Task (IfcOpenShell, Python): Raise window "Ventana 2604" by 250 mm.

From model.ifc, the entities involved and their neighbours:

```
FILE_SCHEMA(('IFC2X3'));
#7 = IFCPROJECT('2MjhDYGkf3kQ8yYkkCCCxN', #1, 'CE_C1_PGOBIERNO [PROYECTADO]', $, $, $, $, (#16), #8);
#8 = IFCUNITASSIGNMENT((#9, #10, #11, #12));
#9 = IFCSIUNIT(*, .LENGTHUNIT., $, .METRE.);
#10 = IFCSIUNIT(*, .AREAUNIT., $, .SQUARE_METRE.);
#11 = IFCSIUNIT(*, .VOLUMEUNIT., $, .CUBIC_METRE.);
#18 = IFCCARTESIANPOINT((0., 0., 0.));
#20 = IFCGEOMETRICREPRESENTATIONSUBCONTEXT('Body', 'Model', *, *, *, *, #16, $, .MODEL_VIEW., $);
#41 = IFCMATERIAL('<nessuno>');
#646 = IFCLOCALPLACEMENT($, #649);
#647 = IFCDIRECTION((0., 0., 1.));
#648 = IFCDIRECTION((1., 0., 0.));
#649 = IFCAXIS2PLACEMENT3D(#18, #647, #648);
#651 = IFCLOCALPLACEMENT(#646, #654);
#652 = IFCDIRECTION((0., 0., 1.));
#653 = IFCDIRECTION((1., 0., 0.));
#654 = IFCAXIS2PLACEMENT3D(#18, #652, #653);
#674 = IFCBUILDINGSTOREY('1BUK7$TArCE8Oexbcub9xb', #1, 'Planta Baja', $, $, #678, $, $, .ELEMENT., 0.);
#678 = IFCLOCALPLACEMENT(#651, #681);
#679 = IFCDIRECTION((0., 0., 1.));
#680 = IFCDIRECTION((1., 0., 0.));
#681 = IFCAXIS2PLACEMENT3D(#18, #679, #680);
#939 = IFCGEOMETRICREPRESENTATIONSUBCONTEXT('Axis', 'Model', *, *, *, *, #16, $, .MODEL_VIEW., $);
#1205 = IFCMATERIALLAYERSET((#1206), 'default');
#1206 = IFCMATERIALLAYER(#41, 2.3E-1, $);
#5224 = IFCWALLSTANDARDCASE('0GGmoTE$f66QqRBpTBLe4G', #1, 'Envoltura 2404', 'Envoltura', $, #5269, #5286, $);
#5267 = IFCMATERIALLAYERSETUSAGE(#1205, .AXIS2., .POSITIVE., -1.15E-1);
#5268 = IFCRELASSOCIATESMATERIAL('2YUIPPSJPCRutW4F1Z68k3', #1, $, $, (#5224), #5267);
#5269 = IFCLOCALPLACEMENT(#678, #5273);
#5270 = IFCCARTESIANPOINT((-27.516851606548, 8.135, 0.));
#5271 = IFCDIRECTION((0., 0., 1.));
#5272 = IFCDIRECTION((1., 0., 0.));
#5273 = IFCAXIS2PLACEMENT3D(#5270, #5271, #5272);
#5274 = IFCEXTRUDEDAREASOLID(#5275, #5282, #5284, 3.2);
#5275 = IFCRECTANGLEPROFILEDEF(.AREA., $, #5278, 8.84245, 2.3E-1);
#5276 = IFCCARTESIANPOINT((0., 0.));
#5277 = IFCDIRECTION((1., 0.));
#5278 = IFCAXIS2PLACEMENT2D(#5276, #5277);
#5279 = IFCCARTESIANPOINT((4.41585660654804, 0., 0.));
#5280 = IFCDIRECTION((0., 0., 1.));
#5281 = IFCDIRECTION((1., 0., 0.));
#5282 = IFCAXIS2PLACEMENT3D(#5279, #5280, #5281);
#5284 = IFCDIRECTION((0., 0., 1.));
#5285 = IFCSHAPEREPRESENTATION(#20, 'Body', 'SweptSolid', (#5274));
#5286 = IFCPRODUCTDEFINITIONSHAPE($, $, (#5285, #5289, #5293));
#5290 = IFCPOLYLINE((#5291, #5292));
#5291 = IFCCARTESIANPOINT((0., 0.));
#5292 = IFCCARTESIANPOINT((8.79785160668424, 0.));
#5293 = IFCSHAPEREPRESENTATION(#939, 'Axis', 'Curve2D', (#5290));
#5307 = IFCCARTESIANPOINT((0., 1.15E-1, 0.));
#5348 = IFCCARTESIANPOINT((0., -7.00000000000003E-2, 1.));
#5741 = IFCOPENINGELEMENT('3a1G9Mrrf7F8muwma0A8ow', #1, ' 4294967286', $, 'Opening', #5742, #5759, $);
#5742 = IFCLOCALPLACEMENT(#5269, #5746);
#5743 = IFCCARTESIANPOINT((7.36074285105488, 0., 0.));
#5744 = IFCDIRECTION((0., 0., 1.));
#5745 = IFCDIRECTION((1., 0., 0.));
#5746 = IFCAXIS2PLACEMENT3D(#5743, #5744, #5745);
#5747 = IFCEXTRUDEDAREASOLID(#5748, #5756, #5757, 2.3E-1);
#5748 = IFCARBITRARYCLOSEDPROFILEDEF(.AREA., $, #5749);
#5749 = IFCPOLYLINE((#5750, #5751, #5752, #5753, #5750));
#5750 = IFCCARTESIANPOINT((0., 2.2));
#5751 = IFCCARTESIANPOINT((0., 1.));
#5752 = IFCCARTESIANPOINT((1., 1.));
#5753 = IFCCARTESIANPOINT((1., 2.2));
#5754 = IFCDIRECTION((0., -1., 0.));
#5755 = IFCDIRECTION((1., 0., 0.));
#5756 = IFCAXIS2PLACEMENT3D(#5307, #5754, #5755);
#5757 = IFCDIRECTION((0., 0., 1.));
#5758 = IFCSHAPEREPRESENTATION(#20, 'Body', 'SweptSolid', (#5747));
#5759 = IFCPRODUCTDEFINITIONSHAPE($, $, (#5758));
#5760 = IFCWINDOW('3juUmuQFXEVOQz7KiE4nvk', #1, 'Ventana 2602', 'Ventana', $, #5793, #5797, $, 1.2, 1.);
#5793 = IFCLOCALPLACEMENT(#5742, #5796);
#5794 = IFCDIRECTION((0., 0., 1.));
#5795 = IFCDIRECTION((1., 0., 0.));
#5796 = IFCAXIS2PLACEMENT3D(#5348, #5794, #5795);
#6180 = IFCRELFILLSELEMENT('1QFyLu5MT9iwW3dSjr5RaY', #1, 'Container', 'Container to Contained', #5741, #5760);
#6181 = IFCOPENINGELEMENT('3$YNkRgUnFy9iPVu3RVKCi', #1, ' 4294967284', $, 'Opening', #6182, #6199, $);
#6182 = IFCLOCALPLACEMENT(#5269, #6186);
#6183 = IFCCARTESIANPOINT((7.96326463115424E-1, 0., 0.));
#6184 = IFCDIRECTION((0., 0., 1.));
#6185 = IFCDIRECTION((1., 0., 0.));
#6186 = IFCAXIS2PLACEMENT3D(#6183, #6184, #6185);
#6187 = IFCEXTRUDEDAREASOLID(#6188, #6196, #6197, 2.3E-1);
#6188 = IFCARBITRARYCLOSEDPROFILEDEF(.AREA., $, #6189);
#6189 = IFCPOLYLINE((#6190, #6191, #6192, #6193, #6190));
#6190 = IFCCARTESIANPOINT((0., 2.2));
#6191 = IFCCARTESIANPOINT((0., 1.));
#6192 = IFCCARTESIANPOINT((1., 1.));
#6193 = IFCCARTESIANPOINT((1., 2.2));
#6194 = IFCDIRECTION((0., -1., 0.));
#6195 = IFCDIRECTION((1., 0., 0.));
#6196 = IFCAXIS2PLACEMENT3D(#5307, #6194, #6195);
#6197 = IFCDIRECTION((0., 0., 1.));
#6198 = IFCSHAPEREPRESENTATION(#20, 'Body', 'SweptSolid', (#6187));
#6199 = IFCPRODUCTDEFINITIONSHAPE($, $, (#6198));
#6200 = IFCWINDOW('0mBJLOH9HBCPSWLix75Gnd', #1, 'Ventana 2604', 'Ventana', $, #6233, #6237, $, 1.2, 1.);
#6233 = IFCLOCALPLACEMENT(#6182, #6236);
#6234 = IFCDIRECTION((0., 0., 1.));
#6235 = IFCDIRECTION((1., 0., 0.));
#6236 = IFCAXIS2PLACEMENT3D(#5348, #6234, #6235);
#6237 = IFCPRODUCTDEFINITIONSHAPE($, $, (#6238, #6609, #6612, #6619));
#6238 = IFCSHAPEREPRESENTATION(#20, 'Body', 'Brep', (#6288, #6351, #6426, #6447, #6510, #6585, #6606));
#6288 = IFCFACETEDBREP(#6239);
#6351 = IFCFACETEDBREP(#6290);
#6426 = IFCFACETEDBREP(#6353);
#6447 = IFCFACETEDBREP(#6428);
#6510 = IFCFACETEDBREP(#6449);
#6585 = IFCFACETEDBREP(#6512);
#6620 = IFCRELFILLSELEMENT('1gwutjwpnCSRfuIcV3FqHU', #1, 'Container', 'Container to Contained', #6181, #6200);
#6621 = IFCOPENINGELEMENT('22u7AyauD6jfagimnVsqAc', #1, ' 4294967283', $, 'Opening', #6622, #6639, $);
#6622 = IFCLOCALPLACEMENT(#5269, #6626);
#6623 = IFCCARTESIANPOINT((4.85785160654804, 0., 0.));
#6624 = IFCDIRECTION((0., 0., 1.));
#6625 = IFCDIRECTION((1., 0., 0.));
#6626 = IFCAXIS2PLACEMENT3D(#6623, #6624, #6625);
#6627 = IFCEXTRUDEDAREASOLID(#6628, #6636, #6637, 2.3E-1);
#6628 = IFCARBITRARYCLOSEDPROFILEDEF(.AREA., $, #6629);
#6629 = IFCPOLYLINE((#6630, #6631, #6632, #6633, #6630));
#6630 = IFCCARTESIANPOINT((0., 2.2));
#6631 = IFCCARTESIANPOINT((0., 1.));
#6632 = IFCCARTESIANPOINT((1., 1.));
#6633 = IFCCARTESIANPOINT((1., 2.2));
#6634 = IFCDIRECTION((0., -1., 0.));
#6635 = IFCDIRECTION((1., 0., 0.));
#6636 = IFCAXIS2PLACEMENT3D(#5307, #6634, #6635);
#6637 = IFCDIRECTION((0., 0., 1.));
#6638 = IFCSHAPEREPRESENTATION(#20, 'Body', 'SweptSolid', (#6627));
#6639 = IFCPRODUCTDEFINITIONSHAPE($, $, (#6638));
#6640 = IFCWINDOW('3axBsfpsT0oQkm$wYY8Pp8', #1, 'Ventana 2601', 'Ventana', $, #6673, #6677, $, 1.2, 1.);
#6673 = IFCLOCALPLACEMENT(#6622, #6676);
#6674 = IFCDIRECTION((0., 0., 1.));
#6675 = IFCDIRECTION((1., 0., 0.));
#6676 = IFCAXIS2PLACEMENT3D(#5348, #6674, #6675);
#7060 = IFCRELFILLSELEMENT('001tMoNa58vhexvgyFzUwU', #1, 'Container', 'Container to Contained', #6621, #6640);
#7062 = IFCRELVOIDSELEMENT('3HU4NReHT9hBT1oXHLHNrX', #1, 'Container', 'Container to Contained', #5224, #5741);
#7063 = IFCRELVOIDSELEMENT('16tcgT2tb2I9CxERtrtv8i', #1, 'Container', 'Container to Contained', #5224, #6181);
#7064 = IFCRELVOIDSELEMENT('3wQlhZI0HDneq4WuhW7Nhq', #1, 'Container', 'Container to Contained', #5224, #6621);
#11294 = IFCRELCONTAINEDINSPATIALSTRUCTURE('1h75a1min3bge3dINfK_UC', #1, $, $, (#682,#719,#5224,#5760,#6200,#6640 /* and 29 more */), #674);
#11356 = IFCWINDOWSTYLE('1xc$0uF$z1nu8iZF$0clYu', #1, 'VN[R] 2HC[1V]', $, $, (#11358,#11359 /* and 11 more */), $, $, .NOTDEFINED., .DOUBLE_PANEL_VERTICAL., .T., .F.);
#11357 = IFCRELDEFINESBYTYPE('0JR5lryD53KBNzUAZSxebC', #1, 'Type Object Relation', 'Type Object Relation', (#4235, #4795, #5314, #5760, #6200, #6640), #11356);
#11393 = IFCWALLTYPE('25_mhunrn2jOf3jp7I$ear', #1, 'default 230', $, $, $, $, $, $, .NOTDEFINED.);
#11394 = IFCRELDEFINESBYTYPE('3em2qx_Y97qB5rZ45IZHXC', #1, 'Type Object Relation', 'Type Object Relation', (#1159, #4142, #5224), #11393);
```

```python
import numpy as np
import ifcopenshell
import ifcopenshell.api.geometry
import ifcopenshell.util.placement
import ifcopenshell.util.unit

model = ifcopenshell.open("model.ifc")
unit_scale = ifcopenshell.util.unit.calculate_unit_scale(model)

window = model.by_guid("0mBJLOH9HBCPSWLix75Gnd")
opening = window.FillsVoids[0].RelatingOpeningElement
dz = 0.25

shift = np.array([0.0, 0.0, dz])
# The window is placed relative to its opening, so it follows when the opening moves.
matrix = ifcopenshell.util.placement.get_local_placement(opening.ObjectPlacement)
matrix[:3, 3] += shift
ifcopenshell.api.geometry.edit_object_placement(
    model, product=opening, matrix=matrix, is_si=False, should_transform_children=True
)

print(f"moved by {dz * unit_scale:+.3f} m")

model.write("model_rev.ifc")
```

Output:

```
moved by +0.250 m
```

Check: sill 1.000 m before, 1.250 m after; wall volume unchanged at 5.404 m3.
